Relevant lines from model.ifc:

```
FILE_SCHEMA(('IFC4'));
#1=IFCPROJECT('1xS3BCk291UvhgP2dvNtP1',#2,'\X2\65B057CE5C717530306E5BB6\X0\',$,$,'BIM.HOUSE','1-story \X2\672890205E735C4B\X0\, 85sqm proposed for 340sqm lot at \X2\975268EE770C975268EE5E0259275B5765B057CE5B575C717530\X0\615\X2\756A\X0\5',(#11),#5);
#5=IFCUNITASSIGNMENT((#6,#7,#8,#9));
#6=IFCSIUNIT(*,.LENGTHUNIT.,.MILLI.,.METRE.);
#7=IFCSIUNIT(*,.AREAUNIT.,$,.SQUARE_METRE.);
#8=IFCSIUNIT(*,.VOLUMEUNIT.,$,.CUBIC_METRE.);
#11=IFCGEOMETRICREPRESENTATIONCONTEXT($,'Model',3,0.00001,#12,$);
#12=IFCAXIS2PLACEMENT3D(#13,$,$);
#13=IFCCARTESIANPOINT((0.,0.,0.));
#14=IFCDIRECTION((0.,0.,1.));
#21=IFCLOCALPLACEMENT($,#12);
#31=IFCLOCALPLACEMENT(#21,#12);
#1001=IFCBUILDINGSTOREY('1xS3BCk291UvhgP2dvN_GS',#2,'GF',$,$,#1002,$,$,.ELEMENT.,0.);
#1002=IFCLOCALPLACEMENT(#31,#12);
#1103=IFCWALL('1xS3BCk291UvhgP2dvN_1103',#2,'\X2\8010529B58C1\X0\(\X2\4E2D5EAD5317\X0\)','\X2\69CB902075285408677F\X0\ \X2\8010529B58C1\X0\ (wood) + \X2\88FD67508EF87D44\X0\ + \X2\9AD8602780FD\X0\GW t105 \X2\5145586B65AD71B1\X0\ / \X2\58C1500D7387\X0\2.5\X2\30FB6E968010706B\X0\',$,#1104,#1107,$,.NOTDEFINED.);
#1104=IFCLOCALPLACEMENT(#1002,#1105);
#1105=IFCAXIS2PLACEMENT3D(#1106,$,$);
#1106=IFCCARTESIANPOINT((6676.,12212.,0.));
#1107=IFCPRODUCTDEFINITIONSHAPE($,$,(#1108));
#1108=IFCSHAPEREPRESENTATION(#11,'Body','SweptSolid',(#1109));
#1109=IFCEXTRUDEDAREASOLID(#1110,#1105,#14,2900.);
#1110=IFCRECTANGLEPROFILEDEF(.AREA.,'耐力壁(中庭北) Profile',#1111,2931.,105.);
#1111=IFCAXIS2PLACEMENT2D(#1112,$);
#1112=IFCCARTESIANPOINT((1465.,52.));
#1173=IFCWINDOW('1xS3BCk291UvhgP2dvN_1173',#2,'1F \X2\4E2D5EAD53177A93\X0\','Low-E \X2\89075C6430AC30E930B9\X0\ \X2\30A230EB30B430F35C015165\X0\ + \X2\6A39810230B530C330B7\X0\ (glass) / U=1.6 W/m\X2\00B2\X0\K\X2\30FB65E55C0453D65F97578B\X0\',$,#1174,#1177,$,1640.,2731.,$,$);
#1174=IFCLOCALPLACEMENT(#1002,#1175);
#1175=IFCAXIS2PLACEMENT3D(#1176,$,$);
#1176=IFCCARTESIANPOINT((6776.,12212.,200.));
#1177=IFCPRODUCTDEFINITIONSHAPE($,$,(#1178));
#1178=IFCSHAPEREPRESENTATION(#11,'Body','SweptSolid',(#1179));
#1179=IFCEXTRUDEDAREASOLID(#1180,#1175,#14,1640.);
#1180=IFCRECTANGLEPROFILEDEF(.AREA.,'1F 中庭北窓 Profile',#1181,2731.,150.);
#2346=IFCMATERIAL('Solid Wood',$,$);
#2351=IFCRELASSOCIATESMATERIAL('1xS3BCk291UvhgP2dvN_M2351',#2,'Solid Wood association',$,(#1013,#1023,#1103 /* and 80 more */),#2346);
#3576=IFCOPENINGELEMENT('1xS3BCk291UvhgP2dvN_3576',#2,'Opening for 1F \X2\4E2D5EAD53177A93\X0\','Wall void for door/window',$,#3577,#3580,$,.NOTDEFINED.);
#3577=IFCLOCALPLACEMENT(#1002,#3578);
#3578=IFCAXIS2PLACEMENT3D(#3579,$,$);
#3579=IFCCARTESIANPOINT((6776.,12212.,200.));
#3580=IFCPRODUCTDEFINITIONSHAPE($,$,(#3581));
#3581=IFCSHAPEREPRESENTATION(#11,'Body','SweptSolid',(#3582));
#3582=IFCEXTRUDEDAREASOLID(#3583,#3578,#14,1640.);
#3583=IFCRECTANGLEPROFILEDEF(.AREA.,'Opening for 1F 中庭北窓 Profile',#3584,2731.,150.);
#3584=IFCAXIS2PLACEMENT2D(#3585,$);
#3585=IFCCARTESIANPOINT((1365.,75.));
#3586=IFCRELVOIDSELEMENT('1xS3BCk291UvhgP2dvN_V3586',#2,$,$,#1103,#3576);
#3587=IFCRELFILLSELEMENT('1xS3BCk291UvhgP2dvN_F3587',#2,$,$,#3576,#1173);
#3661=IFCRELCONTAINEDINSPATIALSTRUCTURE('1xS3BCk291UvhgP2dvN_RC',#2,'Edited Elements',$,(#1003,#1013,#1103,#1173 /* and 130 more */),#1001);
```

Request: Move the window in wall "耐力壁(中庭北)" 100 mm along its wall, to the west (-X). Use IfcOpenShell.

```python
import ifcopenshell
import ifcopenshell.api.geometry
import ifcopenshell.util.placement
import ifcopenshell.util.unit

model = ifcopenshell.open("model.ifc")
unit_scale = ifcopenshell.util.unit.calculate_unit_scale(model)

window = model.by_guid("1xS3BCk291UvhgP2dvN_1173")
opening = window.FillsVoids[0].RelatingOpeningElement
wall = opening.VoidsElements[0].RelatingBuildingElement

wall_matrix = ifcopenshell.util.placement.get_local_placement(wall.ObjectPlacement)
shift = wall_matrix[:3, 0] * -0.1 / unit_scale
before = ifcopenshell.util.placement.get_local_placement(window.ObjectPlacement)[:3, 3].copy()

# The window is not placed relative to its opening, so move both.
for product in (opening, window):
    matrix = ifcopenshell.util.placement.get_local_placement(product.ObjectPlacement)
    matrix[:3, 3] += shift
    ifcopenshell.api.geometry.edit_object_placement(model, product=product, matrix=matrix, is_si=False)

after = ifcopenshell.util.placement.get_local_placement(window.ObjectPlacement)[:3, 3]
print("window moved by", (after - before).round(3) + 0.0)

model.write("model_updated.ifc")
```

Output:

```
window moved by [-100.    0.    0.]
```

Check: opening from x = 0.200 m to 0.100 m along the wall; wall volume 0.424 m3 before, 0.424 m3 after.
